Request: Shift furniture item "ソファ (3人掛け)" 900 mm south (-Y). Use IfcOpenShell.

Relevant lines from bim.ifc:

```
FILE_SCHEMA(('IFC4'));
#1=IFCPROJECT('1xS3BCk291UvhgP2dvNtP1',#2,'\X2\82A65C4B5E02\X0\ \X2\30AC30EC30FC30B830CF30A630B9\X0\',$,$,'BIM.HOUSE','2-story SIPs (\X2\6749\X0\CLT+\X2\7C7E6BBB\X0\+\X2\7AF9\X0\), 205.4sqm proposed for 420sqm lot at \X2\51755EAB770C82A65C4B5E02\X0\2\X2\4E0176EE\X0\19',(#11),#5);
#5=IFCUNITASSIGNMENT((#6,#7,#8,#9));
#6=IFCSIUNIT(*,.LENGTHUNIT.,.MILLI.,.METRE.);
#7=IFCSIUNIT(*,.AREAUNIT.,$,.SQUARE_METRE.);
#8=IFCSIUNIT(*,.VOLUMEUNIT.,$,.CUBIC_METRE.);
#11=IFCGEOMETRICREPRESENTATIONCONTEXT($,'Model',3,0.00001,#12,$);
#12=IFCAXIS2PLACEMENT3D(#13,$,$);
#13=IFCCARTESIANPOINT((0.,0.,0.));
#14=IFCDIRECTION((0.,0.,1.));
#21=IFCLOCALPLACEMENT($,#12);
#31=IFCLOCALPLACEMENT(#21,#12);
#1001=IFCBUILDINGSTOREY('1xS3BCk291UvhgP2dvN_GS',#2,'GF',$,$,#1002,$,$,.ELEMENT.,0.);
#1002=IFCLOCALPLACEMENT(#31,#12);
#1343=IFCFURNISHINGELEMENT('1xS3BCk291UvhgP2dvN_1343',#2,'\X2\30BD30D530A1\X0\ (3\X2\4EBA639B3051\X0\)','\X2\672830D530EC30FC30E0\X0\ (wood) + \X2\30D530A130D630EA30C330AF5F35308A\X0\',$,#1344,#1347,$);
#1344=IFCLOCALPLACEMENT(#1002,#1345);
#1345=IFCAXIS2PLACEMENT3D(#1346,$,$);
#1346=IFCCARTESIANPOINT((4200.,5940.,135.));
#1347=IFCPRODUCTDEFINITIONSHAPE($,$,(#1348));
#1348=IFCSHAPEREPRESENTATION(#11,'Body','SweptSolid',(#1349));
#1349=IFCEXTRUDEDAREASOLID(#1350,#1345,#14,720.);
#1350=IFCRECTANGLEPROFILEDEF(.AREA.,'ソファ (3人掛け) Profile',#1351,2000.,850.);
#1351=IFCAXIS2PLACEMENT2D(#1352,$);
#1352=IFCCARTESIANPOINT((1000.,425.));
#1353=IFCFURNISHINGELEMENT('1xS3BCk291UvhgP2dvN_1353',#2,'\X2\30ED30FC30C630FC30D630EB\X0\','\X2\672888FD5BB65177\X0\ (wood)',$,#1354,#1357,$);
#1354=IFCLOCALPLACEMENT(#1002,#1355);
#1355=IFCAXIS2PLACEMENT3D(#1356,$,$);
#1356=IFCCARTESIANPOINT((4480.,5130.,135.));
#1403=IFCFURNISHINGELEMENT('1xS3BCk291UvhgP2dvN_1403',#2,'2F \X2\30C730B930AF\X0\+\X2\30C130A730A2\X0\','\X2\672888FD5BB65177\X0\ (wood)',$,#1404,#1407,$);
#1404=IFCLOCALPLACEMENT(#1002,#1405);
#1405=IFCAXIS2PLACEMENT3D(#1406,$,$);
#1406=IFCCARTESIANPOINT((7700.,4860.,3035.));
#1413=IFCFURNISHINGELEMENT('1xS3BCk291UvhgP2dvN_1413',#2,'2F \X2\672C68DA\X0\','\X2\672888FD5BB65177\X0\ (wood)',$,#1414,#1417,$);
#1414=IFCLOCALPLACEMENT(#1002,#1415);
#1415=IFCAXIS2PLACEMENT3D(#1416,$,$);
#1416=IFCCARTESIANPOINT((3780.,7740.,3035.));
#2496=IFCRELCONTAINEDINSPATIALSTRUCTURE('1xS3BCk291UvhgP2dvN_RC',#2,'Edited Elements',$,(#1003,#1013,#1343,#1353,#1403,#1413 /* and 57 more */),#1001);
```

```python
import ifcopenshell
import ifcopenshell.api.geometry
import ifcopenshell.util.placement

model = ifcopenshell.open("bim.ifc")

item = model.by_id(1343)
matrix = ifcopenshell.util.placement.get_local_placement(item.ObjectPlacement)
matrix[1, 3] -= 900.0
ifcopenshell.api.geometry.edit_object_placement(model, product=item, matrix=matrix, is_si=False)

print(ifcopenshell.util.placement.get_local_placement(item.ObjectPlacement).round(3) + 0.0)

model.write("bim-out.ifc")
```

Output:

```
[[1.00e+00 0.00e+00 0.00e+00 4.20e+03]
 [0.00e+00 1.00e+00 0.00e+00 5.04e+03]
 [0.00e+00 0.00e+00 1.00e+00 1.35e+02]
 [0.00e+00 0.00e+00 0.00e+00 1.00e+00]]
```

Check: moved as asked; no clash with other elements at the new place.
